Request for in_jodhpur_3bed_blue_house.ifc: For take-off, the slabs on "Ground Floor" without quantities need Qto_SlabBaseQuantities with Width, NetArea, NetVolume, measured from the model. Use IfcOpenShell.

First a look at what the model holds.

```python
import ifcopenshell
import ifcopenshell.util.element
import ifcopenshell.util.unit

model = ifcopenshell.open("in_jodhpur_3bed_blue_house.ifc")
print(model.schema)
for unit_type in ("LENGTHUNIT", "AREAUNIT", "VOLUMEUNIT"):
    print(unit_type, ifcopenshell.util.unit.calculate_unit_scale(model, unit_type))
storey = next(s for s in model.by_type("IfcBuildingStorey") if s.Name == "Ground Floor")
slabs = [e for e in ifcopenshell.util.element.get_decomposition(storey) if e.is_a("IfcSlab")]
for e in sorted(slabs, key=lambda e: e.id()):
    print(e.id(), e.is_a(), e.Name, list(ifcopenshell.util.element.get_psets(e, qtos_only=True)), sep=" | ")
```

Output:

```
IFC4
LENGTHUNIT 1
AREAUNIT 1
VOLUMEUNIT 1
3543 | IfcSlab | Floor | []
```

```python
import ifcopenshell
import ifcopenshell.api.pset
import ifcopenshell.geom
import ifcopenshell.util.element
import ifcopenshell.util.shape
import ifcopenshell.util.unit

model = ifcopenshell.open("in_jodhpur_3bed_blue_house.ifc")
unit_scale = ifcopenshell.util.unit.calculate_unit_scale(model)
area_scale = ifcopenshell.util.unit.calculate_unit_scale(model, "AREAUNIT")
volume_scale = ifcopenshell.util.unit.calculate_unit_scale(model, "VOLUMEUNIT")
settings = ifcopenshell.geom.settings()

storey = next(s for s in model.by_type("IfcBuildingStorey") if s.Name == "Ground Floor")
slabs = [e for e in ifcopenshell.util.element.get_decomposition(storey) if e.is_a("IfcSlab")]

for e in sorted(slabs, key=lambda e: e.id()):
    if ifcopenshell.util.element.get_psets(e, qtos_only=True, should_inherit=False):
        continue
    # Geometry comes back in metres, in the element's own axes.
    shape = ifcopenshell.geom.create_shape(settings, e)
    values = {
        "Width": ifcopenshell.util.shape.get_z(shape.geometry) / unit_scale,
        "NetArea": ifcopenshell.util.shape.get_footprint_area(shape.geometry) / area_scale,
        "NetVolume": ifcopenshell.util.shape.get_volume(shape.geometry) / volume_scale,
    }
    qto = ifcopenshell.api.pset.add_qto(model, product=e, name="Qto_SlabBaseQuantities")
    ifcopenshell.api.pset.edit_qto(model, qto=qto, properties=values)
    print(e.id(), {k: round(v, 3) for k, v in values.items()})

model.write("in_jodhpur_3bed_blue_house_edited.ifc")
```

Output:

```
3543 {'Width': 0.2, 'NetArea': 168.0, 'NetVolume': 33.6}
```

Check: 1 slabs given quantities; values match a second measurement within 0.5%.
